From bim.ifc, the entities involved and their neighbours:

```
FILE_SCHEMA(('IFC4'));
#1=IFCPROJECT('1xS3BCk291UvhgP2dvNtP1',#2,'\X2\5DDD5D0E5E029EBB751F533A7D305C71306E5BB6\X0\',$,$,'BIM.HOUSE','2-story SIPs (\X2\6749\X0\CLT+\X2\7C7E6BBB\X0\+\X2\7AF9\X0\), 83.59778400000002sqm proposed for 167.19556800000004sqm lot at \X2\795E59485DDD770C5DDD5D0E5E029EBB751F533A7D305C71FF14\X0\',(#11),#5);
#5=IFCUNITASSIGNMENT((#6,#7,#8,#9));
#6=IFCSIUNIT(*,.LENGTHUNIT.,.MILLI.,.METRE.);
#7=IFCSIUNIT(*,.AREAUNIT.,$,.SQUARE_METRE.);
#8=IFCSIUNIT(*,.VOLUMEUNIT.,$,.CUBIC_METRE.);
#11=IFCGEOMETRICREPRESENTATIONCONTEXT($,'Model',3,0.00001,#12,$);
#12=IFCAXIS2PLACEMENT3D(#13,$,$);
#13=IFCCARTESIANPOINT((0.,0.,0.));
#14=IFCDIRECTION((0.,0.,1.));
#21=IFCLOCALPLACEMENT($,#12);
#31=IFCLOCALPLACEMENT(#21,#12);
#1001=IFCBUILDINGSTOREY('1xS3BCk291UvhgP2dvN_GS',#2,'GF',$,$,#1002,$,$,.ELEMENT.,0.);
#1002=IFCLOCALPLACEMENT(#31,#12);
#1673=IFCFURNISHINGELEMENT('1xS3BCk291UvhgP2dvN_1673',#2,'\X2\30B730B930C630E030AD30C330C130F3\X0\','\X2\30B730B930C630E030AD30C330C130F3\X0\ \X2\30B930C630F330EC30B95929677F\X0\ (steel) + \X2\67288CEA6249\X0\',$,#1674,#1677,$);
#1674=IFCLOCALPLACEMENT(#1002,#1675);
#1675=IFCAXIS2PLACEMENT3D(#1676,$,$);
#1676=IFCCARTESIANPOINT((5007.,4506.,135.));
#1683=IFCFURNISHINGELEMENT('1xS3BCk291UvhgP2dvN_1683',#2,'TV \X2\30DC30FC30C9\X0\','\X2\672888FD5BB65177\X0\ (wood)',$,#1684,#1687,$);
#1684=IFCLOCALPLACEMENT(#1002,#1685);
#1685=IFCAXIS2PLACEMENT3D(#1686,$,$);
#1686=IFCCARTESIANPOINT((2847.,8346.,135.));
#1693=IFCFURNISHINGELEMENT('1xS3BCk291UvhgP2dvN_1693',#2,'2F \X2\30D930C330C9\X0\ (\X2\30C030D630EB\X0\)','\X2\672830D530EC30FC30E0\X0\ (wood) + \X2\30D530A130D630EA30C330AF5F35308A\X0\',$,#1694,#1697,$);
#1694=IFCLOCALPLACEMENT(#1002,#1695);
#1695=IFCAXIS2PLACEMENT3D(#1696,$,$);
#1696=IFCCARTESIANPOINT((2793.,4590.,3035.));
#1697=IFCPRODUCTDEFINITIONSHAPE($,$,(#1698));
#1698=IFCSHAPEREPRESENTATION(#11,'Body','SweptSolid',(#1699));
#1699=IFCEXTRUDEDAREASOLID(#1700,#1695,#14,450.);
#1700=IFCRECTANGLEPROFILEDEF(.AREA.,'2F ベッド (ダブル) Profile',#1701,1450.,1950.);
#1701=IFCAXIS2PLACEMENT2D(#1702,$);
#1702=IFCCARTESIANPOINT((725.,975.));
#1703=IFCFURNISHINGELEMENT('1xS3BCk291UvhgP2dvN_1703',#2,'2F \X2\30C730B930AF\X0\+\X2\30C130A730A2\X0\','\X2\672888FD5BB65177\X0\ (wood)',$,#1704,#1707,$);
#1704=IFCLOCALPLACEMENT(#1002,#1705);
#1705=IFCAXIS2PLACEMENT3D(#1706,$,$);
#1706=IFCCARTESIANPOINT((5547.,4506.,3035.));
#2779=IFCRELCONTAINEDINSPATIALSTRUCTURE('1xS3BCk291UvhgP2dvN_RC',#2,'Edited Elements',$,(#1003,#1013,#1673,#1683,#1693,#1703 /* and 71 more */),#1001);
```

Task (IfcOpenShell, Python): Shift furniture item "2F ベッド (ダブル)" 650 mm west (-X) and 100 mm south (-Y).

```python
import ifcopenshell
import ifcopenshell.api.geometry
import ifcopenshell.util.placement
import ifcopenshell.util.unit

model = ifcopenshell.open("bim.ifc")
unit_scale = ifcopenshell.util.unit.calculate_unit_scale(model)

item = model.by_guid("1xS3BCk291UvhgP2dvN_1693")
matrix = ifcopenshell.util.placement.get_local_placement(item.ObjectPlacement)
matrix[0, 3] -= 0.65 / unit_scale
matrix[1, 3] -= 0.1 / unit_scale
ifcopenshell.api.geometry.edit_object_placement(model, product=item, matrix=matrix, is_si=False)

print(ifcopenshell.util.placement.get_local_placement(item.ObjectPlacement).round(3) + 0.0)

model.write("bim_edited.ifc")
```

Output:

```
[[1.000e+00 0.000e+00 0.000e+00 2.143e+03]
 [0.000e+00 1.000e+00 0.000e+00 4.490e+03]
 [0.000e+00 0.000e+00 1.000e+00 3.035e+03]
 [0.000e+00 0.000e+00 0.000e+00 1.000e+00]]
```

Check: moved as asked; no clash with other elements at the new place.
